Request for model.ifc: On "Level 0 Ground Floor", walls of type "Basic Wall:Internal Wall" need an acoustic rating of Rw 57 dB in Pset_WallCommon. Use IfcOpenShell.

First a look at what the model holds.

```python
import ifcopenshell
import ifcopenshell.util.element

model = ifcopenshell.open("model.ifc")
print(model.schema)
storey = next(s for s in model.by_type("IfcBuildingStorey") if s.Name == "Level 0 Ground Floor")
walls = [e for e in ifcopenshell.util.element.get_decomposition(storey) if e.is_a("IfcWall")]
seen = {}
for e in walls:
    element_type = ifcopenshell.util.element.get_type(e)
    key = (element_type.Name if element_type != e and element_type else None, ifcopenshell.util.element.get_pset(e, "Pset_WallCommon", "AcousticRating"))
    seen[key] = seen.get(key, 0) + 1
for (name, value), count in sorted(seen.items(), key=str):
    print(count, "x", name, "|", value)
```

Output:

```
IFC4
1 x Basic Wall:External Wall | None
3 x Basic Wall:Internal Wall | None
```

```python
import ifcopenshell
import ifcopenshell.api.pset
import ifcopenshell.util.element

model = ifcopenshell.open("model.ifc")

storey = next(s for s in model.by_type("IfcBuildingStorey") if s.Name == "Level 0 Ground Floor")
walls = [e for e in ifcopenshell.util.element.get_decomposition(storey) if e.is_a("IfcWall")]

count = 0
for e in walls:
    element_type = ifcopenshell.util.element.get_type(e)
    if element_type in (None, e) or element_type.Name != "Basic Wall:Internal Wall":
        continue
    # add_pset returns the element's existing set when there is one.
    pset = ifcopenshell.api.pset.add_pset(model, product=e, name="Pset_WallCommon")
    ifcopenshell.api.pset.edit_pset(model, pset=pset, properties={"AcousticRating": "Rw 57 dB"})
    count += 1

print(count, "walls updated")

model.write("model_rev.ifc")
```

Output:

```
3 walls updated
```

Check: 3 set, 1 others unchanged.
